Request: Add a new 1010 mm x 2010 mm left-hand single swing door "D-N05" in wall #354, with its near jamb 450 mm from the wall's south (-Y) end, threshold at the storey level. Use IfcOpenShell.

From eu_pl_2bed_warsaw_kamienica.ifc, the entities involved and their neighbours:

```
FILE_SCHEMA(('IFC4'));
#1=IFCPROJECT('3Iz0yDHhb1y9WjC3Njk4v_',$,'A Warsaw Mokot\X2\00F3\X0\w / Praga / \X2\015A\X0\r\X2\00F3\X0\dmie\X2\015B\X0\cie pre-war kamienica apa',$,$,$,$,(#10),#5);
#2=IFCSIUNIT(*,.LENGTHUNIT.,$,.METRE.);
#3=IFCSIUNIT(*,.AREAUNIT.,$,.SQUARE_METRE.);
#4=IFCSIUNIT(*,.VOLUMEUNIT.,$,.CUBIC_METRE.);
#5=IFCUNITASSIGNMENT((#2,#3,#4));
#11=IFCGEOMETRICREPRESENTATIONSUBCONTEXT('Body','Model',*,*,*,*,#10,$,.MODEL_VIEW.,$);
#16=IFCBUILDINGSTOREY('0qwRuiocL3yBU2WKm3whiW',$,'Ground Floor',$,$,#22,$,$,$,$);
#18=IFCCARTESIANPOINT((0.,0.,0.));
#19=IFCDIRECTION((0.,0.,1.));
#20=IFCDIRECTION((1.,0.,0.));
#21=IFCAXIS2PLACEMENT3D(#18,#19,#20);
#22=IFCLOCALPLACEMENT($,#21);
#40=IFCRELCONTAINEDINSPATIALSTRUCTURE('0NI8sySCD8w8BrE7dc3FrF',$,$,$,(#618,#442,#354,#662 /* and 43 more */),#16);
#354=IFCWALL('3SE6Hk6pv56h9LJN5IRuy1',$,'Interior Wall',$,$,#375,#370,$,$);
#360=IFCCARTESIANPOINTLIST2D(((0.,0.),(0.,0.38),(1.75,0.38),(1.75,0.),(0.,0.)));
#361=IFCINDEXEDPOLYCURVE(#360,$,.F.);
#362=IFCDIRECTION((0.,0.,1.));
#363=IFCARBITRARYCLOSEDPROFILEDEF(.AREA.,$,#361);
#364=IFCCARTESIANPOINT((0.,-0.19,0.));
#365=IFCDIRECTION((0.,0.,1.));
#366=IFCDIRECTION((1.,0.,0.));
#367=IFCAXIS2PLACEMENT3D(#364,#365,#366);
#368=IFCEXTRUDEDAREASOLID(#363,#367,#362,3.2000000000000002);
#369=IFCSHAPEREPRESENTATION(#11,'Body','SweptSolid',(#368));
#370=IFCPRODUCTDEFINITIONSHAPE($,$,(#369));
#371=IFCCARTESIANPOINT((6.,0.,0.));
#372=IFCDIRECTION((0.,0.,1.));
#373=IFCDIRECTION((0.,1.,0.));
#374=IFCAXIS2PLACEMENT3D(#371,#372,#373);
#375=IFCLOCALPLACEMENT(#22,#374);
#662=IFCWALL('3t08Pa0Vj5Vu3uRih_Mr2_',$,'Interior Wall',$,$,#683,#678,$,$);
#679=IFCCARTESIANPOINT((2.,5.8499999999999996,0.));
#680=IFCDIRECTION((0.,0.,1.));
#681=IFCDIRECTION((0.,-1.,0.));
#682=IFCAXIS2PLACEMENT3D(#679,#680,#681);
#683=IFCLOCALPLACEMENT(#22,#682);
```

```python
import numpy as np
import ifcopenshell
import ifcopenshell.api.feature
import ifcopenshell.api.geometry
import ifcopenshell.api.root
import ifcopenshell.api.spatial
import ifcopenshell.geom
import ifcopenshell.util.element
import ifcopenshell.util.placement
import ifcopenshell.util.representation
import ifcopenshell.util.shape
import ifcopenshell.util.unit

model = ifcopenshell.open("eu_pl_2bed_warsaw_kamienica.ifc")
unit_scale = ifcopenshell.util.unit.calculate_unit_scale(model)
settings = ifcopenshell.geom.settings()


def volume(element):
    """Net volume in cubic metres, openings subtracted."""
    shape = ifcopenshell.geom.create_shape(settings, element)
    return ifcopenshell.util.shape.get_volume(shape.geometry)


wall = model.by_id(354)
storey = ifcopenshell.util.element.get_container(wall, ifc_class="IfcBuildingStorey")
context = ifcopenshell.util.representation.get_context(model, "Model", "Body", "MODEL_VIEW")
before = volume(wall)

width, height, from_end, sill = 1.01, 2.01, 0.45, 0.0  # metres

# The wall runs along its own X axis, and the end named is its -X end.
wall_shape = ifcopenshell.geom.create_shape(settings, wall)
x, y, z = ifcopenshell.util.shape.get_vertices(wall_shape.geometry).T
start = x.min() + from_end
face, thickness = float(y.min()), float(y.max() - y.min())
wall_matrix = ifcopenshell.util.placement.get_local_placement(wall.ObjectPlacement)
level = ifcopenshell.util.placement.get_local_placement(storey.ObjectPlacement)[2, 3]


def in_wall(x, y):
    """Placement at x, y metres in the wall's axes, at sill height."""
    matrix = wall_matrix.copy()
    matrix[:, 3] = wall_matrix @ np.array([x / unit_scale, y / unit_scale, 0.0, 1.0])
    matrix[2, 3] = level + sill / unit_scale
    return matrix


# Opening: a box that overshoots both wall faces by 50 mm.
opening = ifcopenshell.api.root.create_entity(model, ifc_class="IfcOpeningElement", predefined_type="OPENING")
box = ifcopenshell.api.geometry.add_wall_representation(
    model, context=context, length=width, height=height, thickness=thickness + 0.1
)
ifcopenshell.api.geometry.assign_representation(model, product=opening, representation=box)
ifcopenshell.api.geometry.edit_object_placement(model, product=opening, matrix=in_wall(start, face - 0.05), is_si=False)
ifcopenshell.api.feature.add_feature(model, feature=opening, element=wall)

door = ifcopenshell.api.root.create_entity(model, ifc_class="IfcDoor", name="D-N05", predefined_type="DOOR")
door.OverallWidth, door.OverallHeight = width / unit_scale, height / unit_scale
door.OperationType = "SINGLE_SWING_LEFT"
body = ifcopenshell.api.geometry.add_door_representation(
    model,
    context=context,
    overall_width=door.OverallWidth,
    overall_height=door.OverallHeight,
    operation_type="SINGLE_SWING_LEFT",
    lining_properties={"LiningDepth": thickness / unit_scale, "ThresholdDepth": thickness / unit_scale},
)
ifcopenshell.api.geometry.assign_representation(model, product=door, representation=body)
ifcopenshell.api.spatial.assign_container(model, products=[door], relating_structure=storey)
ifcopenshell.api.feature.add_filling(model, opening=opening, element=door)

# The lining spans the wall, so the door starts at the wall face.
ifcopenshell.api.geometry.edit_object_placement(model, product=door, matrix=in_wall(start, face), is_si=False)

after = volume(wall)

print(f"wall volume {before:.3f} -> {after:.3f} m3")

model.write("eu_pl_2bed_warsaw_kamienica_rev.ifc")
```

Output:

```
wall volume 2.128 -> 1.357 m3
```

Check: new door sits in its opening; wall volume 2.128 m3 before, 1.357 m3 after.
